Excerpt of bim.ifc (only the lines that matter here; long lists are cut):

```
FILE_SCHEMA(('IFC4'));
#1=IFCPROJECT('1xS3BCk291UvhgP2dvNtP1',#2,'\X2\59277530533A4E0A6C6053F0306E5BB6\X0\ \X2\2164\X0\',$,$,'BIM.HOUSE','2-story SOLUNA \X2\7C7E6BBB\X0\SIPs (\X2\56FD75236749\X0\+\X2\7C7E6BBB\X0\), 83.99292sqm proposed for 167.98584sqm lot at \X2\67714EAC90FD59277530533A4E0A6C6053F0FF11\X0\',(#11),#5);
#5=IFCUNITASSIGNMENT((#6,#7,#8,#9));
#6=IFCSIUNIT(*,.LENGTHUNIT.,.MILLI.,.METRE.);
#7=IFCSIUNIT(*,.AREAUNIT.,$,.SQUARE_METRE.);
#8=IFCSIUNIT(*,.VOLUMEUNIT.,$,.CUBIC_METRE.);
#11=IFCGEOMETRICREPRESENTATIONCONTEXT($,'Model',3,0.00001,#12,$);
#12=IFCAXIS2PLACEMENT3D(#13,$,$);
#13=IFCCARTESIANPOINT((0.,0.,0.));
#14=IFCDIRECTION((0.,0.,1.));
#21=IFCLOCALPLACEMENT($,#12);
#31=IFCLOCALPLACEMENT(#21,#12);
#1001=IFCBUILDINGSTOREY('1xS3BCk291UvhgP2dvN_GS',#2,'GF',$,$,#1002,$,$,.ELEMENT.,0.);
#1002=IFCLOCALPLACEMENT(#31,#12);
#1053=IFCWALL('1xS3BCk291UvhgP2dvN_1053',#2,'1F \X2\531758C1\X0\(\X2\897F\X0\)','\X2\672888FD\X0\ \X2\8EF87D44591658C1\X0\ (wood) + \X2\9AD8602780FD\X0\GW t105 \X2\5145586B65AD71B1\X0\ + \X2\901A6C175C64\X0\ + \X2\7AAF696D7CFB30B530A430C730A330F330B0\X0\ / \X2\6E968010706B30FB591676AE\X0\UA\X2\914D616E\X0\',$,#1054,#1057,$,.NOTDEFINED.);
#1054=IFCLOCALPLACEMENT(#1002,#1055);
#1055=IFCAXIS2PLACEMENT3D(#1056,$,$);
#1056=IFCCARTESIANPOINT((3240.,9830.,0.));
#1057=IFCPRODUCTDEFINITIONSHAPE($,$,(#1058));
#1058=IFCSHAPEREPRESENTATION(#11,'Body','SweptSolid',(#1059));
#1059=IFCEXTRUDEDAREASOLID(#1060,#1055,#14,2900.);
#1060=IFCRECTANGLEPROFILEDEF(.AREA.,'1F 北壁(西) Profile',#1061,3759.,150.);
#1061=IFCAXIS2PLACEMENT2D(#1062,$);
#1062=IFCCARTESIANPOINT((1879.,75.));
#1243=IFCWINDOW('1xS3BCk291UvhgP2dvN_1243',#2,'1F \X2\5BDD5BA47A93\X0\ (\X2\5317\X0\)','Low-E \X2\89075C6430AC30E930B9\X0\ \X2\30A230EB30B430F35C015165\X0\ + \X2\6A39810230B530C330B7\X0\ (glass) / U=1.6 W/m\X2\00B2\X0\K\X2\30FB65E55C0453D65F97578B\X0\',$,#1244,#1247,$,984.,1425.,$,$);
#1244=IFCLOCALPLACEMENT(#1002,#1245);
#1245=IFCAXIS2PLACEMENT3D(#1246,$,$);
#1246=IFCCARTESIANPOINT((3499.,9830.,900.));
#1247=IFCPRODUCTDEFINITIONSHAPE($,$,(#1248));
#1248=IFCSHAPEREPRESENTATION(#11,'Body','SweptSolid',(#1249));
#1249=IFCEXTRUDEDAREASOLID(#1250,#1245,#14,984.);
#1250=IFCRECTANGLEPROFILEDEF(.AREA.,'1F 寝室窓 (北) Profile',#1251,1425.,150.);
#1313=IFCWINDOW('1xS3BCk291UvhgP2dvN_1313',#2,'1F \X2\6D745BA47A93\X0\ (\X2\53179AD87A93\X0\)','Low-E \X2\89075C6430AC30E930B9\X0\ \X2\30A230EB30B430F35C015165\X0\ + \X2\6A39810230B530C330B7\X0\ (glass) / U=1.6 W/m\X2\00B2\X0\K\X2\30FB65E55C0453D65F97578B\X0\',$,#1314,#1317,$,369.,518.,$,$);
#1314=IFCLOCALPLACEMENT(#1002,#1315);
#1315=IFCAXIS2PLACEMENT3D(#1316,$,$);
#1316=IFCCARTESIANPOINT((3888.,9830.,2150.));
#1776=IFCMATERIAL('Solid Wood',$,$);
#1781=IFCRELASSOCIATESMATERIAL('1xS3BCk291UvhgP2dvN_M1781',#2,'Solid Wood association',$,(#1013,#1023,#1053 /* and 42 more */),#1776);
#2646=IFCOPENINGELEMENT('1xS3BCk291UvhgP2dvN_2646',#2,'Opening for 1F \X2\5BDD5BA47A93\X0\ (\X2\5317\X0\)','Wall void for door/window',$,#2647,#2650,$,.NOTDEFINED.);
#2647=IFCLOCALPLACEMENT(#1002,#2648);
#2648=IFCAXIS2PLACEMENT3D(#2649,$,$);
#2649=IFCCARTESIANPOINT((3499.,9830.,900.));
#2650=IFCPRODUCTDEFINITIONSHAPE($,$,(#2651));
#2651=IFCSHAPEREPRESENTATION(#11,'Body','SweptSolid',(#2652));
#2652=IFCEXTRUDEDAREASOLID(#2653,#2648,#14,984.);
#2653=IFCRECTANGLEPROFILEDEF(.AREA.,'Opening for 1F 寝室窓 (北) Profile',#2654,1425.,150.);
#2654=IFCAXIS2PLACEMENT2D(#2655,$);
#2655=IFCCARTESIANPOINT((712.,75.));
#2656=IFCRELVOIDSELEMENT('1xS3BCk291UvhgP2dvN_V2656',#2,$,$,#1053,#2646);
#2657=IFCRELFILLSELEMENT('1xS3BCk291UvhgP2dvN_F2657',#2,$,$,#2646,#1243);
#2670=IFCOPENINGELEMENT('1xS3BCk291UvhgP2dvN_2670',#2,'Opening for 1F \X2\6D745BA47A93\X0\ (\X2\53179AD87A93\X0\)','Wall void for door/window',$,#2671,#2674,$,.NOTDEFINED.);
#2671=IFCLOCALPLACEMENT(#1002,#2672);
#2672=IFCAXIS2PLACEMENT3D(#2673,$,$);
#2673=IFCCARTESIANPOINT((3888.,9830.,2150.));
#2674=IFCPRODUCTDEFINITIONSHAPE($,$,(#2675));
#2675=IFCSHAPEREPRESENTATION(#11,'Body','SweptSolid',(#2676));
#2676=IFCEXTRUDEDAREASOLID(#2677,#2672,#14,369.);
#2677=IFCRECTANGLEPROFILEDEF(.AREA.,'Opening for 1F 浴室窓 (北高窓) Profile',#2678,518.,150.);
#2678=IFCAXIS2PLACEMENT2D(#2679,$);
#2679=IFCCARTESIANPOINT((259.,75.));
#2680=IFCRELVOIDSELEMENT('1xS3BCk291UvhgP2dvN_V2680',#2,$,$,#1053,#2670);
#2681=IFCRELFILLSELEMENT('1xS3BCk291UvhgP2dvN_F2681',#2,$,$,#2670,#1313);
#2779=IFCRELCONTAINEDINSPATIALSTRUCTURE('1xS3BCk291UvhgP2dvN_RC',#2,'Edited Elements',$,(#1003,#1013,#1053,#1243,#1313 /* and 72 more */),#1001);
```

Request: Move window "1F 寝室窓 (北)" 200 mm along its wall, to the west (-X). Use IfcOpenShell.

```python
import ifcopenshell
import ifcopenshell.api.geometry
import ifcopenshell.util.placement
import ifcopenshell.util.unit

model = ifcopenshell.open("bim.ifc")
unit_scale = ifcopenshell.util.unit.calculate_unit_scale(model)

window = model.by_id(1243)
opening = window.FillsVoids[0].RelatingOpeningElement
wall = opening.VoidsElements[0].RelatingBuildingElement

wall_matrix = ifcopenshell.util.placement.get_local_placement(wall.ObjectPlacement)
shift = wall_matrix[:3, 0] * -0.2 / unit_scale
before = ifcopenshell.util.placement.get_local_placement(window.ObjectPlacement)[:3, 3].copy()

# The window is not placed relative to its opening, so move both.
for product in (opening, window):
    matrix = ifcopenshell.util.placement.get_local_placement(product.ObjectPlacement)
    matrix[:3, 3] += shift
    ifcopenshell.api.geometry.edit_object_placement(model, product=product, matrix=matrix, is_si=False)

after = ifcopenshell.util.placement.get_local_placement(window.ObjectPlacement)[:3, 3]
print("window moved by", (after - before).round(3) + 0.0)

model.write("bim_edited.ifc")
```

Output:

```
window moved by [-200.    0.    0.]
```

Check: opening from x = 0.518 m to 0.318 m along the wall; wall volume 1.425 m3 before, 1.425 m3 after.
